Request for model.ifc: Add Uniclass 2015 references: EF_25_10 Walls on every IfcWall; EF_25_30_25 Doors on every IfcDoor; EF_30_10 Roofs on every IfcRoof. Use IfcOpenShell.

First a look at what the model holds.

```python
import ifcopenshell

model = ifcopenshell.open("model.ifc")
print(model.schema)
print("classifications:", [c.Name for c in model.by_type("IfcClassification")])
for ifc_class in ("IfcDoor", "IfcRoof", "IfcStair", "IfcWall", "IfcWindow"):
    print(ifc_class, len(model.by_type(ifc_class)))
```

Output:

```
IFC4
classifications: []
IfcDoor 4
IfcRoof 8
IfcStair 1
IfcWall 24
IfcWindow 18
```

```python
import ifcopenshell
import ifcopenshell.api.classification

model = ifcopenshell.open("model.ifc")

system = ifcopenshell.api.classification.add_classification(model, classification="Uniclass 2015")

codes = {
    "IfcWall": ("EF_25_10", "Walls"),
    "IfcDoor": ("EF_25_30_25", "Doors"),
    "IfcRoof": ("EF_30_10", "Roofs"),
}
for ifc_class, (code, name) in codes.items():
    products = model.by_type(ifc_class)
    ifcopenshell.api.classification.add_reference(
        model, products=products, classification=system, identification=code, name=name
    )
    print(code, len(products))

model.write("model_v2.ifc")
```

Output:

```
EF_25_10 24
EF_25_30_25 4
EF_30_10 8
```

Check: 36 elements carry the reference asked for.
